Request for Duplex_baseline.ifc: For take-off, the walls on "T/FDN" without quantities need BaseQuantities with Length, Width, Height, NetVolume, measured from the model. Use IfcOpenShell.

First a look at what the model holds.

```python
import ifcopenshell
import ifcopenshell.util.element
import ifcopenshell.util.unit

model = ifcopenshell.open("Duplex_baseline.ifc")
print(model.schema)
for unit_type in ("LENGTHUNIT", "AREAUNIT", "VOLUMEUNIT"):
    print(unit_type, ifcopenshell.util.unit.calculate_unit_scale(model, unit_type))
storey = next(s for s in model.by_type("IfcBuildingStorey") if s.Name == "T/FDN")
walls = [e for e in ifcopenshell.util.element.get_decomposition(storey) if e.is_a("IfcWall")]
for e in sorted(walls, key=lambda e: e.id()):
    print(e.id(), e.is_a(), e.Name, list(ifcopenshell.util.element.get_psets(e, qtos_only=True)), sep=" | ")
```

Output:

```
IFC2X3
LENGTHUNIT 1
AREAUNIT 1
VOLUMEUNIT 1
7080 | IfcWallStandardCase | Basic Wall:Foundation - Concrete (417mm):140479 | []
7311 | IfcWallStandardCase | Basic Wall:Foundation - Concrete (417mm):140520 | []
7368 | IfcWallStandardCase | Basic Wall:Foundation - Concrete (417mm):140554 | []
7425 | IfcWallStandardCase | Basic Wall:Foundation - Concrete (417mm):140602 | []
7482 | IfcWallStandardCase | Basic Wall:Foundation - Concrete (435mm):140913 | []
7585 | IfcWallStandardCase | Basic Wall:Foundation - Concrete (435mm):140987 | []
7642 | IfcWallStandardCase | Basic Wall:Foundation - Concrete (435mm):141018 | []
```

```python
import ifcopenshell
import ifcopenshell.api.pset
import ifcopenshell.geom
import ifcopenshell.util.element
import ifcopenshell.util.shape
import ifcopenshell.util.unit

model = ifcopenshell.open("Duplex_baseline.ifc")
unit_scale = ifcopenshell.util.unit.calculate_unit_scale(model)
volume_scale = ifcopenshell.util.unit.calculate_unit_scale(model, "VOLUMEUNIT")
settings = ifcopenshell.geom.settings()

storey = next(s for s in model.by_type("IfcBuildingStorey") if s.Name == "T/FDN")
walls = [e for e in ifcopenshell.util.element.get_decomposition(storey) if e.is_a("IfcWall")]

for e in sorted(walls, key=lambda e: e.id()):
    if ifcopenshell.util.element.get_psets(e, qtos_only=True, should_inherit=False):
        continue
    # Geometry comes back in metres, in the element's own axes.
    shape = ifcopenshell.geom.create_shape(settings, e)
    values = {
        "Length": ifcopenshell.util.shape.get_x(shape.geometry) / unit_scale,
        "Width": ifcopenshell.util.shape.get_y(shape.geometry) / unit_scale,
        "Height": ifcopenshell.util.shape.get_z(shape.geometry) / unit_scale,
        "NetVolume": ifcopenshell.util.shape.get_volume(shape.geometry) / volume_scale,
    }
    qto = ifcopenshell.api.pset.add_qto(model, product=e, name="BaseQuantities")
    ifcopenshell.api.pset.edit_qto(model, qto=qto, properties=values)
    print(e.id(), {k: round(v, 3) for k, v in values.items()})

model.write("Duplex_baseline_edited.ifc")
```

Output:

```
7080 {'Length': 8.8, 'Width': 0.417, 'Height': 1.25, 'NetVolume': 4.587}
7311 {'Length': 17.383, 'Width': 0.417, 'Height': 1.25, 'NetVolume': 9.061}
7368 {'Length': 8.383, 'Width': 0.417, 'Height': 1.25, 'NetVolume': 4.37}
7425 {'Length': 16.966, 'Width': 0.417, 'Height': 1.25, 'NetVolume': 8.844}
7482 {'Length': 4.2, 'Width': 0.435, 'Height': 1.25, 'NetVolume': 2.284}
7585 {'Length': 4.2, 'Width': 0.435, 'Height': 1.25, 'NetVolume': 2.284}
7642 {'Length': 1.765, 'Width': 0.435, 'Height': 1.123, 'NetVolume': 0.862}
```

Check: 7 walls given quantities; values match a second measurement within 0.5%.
